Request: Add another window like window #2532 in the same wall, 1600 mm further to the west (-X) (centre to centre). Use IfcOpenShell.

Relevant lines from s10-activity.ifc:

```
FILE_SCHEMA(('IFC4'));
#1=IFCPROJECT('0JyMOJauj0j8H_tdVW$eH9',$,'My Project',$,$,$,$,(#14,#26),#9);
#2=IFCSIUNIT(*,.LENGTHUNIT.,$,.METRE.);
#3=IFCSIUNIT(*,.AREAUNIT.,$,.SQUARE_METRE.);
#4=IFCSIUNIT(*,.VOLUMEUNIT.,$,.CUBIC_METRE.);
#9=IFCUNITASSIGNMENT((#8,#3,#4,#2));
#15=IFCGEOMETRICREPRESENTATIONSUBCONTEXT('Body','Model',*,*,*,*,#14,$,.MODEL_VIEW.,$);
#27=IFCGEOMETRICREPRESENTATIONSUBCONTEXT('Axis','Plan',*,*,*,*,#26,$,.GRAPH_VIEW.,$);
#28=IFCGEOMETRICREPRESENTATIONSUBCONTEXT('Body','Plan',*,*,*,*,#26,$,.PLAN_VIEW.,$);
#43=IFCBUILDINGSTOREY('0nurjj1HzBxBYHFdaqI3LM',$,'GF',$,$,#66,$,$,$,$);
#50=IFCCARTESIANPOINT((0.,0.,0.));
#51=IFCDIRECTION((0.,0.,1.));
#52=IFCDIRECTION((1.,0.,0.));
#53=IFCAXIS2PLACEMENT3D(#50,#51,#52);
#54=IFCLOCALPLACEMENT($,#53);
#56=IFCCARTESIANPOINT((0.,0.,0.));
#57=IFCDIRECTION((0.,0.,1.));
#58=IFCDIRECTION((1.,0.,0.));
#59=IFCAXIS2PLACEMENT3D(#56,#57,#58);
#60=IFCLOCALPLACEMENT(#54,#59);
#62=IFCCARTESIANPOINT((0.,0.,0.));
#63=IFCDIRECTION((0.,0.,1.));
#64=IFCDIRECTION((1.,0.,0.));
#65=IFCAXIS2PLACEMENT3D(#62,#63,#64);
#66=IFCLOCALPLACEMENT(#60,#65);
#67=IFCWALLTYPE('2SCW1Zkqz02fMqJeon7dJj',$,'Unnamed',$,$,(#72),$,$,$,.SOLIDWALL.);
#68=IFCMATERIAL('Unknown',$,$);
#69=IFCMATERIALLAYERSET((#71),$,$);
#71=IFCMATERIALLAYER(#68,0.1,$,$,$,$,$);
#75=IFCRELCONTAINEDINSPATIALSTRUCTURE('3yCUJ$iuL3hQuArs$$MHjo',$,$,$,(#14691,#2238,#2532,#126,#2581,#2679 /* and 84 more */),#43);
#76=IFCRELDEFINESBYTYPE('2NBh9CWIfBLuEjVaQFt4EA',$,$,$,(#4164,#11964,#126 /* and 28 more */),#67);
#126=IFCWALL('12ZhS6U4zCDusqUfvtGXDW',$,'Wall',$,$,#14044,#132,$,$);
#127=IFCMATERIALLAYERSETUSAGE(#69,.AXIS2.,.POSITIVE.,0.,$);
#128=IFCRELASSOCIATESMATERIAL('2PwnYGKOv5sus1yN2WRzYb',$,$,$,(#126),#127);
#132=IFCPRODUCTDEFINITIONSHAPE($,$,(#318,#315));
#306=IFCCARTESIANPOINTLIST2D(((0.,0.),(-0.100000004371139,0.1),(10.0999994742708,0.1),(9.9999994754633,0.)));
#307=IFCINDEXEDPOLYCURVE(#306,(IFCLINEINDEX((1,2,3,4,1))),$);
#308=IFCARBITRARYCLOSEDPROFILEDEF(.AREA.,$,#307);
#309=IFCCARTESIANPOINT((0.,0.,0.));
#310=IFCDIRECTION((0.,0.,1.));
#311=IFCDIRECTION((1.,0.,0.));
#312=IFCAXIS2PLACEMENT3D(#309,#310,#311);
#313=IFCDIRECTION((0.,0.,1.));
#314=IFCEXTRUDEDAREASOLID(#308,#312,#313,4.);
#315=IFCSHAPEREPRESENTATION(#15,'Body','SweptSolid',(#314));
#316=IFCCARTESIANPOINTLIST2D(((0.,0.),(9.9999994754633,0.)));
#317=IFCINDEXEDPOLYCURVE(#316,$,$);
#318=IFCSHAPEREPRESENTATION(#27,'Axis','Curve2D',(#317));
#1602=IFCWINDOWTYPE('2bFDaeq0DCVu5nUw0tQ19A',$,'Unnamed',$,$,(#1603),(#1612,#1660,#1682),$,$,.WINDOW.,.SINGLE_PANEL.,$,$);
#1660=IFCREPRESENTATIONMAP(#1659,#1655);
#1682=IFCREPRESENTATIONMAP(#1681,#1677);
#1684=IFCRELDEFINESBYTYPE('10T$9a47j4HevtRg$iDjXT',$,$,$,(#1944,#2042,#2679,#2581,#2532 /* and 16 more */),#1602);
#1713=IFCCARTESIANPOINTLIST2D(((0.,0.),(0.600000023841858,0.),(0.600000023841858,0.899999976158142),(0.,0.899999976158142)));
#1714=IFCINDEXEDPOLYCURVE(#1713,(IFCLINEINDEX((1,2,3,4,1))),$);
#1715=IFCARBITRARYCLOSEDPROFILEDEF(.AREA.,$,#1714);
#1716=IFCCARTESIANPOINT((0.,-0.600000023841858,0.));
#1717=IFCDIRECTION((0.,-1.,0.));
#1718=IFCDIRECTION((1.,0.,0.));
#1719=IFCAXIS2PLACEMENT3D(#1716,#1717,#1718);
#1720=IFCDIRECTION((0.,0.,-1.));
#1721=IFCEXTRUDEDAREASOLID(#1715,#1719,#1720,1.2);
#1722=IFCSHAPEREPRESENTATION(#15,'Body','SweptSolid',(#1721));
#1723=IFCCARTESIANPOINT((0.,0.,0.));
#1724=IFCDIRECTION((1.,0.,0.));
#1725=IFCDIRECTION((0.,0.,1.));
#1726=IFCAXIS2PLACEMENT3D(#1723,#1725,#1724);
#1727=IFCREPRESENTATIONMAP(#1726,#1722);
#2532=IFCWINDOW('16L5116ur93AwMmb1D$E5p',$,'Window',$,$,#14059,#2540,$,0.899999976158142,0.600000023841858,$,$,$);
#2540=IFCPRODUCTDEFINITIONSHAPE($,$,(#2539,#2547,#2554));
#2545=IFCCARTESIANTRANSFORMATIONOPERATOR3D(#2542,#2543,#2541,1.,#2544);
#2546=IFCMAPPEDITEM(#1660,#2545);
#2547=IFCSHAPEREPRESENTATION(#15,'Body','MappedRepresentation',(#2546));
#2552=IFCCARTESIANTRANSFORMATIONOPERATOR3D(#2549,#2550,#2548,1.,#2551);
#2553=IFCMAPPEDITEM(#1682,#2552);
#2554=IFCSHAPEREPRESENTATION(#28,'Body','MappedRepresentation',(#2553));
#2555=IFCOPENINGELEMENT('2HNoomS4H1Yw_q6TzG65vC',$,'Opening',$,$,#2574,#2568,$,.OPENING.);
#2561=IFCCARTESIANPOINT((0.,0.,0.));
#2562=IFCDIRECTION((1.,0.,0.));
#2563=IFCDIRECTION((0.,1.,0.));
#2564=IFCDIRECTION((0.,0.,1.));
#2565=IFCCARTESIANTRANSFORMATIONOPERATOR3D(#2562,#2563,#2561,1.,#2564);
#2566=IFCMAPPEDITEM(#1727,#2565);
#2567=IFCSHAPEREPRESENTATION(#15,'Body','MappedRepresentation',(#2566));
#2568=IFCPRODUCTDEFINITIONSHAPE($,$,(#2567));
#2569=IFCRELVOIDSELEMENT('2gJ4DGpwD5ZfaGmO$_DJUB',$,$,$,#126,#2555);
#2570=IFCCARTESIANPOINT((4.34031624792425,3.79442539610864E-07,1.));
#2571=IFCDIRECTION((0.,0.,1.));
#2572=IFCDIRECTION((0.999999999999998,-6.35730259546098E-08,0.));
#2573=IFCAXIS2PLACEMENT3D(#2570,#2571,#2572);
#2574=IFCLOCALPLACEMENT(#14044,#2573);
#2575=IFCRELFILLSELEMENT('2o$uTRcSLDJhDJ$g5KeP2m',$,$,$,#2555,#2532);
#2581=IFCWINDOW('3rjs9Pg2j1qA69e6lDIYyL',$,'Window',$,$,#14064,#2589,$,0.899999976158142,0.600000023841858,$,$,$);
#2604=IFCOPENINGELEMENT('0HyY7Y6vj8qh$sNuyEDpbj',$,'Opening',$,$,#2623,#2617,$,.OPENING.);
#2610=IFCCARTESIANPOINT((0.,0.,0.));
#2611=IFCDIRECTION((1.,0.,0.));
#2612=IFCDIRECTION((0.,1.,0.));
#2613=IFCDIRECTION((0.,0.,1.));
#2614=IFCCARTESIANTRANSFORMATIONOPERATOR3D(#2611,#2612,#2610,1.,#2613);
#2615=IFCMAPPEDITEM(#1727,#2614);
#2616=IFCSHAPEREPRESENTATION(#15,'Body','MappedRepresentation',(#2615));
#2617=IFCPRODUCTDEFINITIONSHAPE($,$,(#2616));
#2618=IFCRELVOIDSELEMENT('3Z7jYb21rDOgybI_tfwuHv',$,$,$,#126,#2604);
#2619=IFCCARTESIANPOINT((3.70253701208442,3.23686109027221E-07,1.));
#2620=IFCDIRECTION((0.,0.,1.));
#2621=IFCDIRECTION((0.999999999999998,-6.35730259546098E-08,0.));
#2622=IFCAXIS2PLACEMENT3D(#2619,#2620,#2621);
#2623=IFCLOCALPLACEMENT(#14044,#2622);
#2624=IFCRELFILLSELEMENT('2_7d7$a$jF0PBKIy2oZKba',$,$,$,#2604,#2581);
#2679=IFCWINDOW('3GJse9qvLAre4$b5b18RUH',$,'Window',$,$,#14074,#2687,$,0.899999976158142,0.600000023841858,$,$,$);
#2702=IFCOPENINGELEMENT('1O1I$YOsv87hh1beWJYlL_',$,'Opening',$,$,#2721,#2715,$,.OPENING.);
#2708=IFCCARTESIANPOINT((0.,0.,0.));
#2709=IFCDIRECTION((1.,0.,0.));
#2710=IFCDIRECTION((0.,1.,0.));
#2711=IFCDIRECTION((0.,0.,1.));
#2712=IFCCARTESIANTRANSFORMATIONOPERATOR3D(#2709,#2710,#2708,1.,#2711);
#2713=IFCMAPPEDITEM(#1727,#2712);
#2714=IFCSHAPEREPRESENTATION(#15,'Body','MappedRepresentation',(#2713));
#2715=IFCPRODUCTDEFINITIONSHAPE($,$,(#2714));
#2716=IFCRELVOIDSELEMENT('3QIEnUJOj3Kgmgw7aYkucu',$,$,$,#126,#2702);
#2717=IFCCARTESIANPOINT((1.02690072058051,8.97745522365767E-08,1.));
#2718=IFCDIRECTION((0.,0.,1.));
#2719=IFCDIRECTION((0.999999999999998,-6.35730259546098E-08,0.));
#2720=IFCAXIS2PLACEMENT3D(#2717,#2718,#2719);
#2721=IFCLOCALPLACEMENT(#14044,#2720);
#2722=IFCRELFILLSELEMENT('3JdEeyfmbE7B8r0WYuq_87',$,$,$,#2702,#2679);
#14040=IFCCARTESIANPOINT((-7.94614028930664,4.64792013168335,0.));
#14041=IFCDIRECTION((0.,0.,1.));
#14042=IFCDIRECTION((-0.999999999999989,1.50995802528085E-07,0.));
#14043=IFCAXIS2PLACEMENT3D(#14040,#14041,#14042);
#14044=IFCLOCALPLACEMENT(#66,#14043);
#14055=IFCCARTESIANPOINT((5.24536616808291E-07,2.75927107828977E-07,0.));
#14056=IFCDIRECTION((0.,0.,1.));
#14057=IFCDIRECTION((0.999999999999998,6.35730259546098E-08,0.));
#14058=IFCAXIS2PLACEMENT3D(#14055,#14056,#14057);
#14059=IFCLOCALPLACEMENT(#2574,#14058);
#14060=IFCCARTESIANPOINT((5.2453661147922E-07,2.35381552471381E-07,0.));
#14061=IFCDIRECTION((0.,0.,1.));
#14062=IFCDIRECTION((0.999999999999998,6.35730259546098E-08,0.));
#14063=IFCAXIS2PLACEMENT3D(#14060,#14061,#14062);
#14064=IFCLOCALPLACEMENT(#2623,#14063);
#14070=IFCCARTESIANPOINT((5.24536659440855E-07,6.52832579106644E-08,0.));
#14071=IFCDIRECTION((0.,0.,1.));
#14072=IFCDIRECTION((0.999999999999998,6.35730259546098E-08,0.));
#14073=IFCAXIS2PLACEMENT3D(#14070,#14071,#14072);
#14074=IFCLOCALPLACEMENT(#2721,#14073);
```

```python
import ifcopenshell
import ifcopenshell.api.feature
import ifcopenshell.api.geometry
import ifcopenshell.api.root
import ifcopenshell.geom
import ifcopenshell.util.element
import ifcopenshell.util.placement
import ifcopenshell.util.shape
import ifcopenshell.util.unit

model = ifcopenshell.open("s10-activity.ifc")
unit_scale = ifcopenshell.util.unit.calculate_unit_scale(model)
settings = ifcopenshell.geom.settings()


def volume(element):
    """Net volume in cubic metres, openings subtracted."""
    shape = ifcopenshell.geom.create_shape(settings, element)
    return ifcopenshell.util.shape.get_volume(shape.geometry)


window = model.by_guid("16L5116ur93AwMmb1D$E5p")
opening = window.FillsVoids[0].RelatingOpeningElement
wall = opening.VoidsElements[0].RelatingBuildingElement
before = volume(wall)
shift = ifcopenshell.util.placement.get_local_placement(wall.ObjectPlacement)[:3, 0] * 1.6 / unit_scale

# copy_class copies the void relationship, type, container and properties, but no geometry.
new_opening = ifcopenshell.api.root.copy_class(model, product=opening)
new_opening.Representation = ifcopenshell.util.element.copy_deep(
    model, opening.Representation, exclude=["IfcGeometricRepresentationContext", "IfcRepresentationMap"]
)
new_window = ifcopenshell.api.root.copy_class(model, product=window)
new_window.Representation = ifcopenshell.util.element.copy_deep(
    model, window.Representation, exclude=["IfcGeometricRepresentationContext", "IfcRepresentationMap"]
)
ifcopenshell.api.feature.add_filling(model, opening=new_opening, element=new_window)

for old, new in ((opening, new_opening), (window, new_window)):
    matrix = ifcopenshell.util.placement.get_local_placement(old.ObjectPlacement)
    matrix[:3, 3] += shift
    ifcopenshell.api.geometry.edit_object_placement(model, product=new, matrix=matrix, is_si=False)

after = volume(wall)

print(f"wall volume {before:.3f} -> {after:.3f} m3")

model.write("s10-activity-out.ifc")
```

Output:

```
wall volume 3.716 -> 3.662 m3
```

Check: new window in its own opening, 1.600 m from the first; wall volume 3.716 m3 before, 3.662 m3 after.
